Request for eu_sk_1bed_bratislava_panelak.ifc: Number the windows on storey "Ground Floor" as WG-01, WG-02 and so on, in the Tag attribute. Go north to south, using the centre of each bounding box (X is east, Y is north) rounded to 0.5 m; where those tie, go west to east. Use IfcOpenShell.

First a look at what the model holds.

```python
import ifcopenshell
import ifcopenshell.util.element
import ifcopenshell.util.placement

model = ifcopenshell.open("eu_sk_1bed_bratislava_panelak.ifc")
print(model.schema)
storey = next(s for s in model.by_type("IfcBuildingStorey") if s.Name == "Ground Floor")
windows = [e for e in ifcopenshell.util.element.get_decomposition(storey) if e.is_a("IfcWindow")]
for e in sorted(windows, key=lambda e: e.id()):
    origin = ifcopenshell.util.placement.get_local_placement(e.ObjectPlacement)[:3, 3]
    print(e.id(), e.Tag, e.Name, origin.round(2) + 0.0, sep=" | ")
```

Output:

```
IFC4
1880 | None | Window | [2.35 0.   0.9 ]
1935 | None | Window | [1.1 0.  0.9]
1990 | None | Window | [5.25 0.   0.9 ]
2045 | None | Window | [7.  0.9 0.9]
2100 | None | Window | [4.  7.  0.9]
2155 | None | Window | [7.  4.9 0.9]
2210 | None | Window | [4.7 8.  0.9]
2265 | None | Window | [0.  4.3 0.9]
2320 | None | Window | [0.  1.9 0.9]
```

```python
import ifcopenshell
import ifcopenshell.geom
import ifcopenshell.util.element
import ifcopenshell.util.shape

model = ifcopenshell.open("eu_sk_1bed_bratislava_panelak.ifc")
settings = ifcopenshell.geom.settings()
settings.set("use-world-coords", True)


def centre(element):
    shape = ifcopenshell.geom.create_shape(settings, element)
    return ifcopenshell.util.shape.get_bbox_centroid(shape.geometry)


storey = next(s for s in model.by_type("IfcBuildingStorey") if s.Name == "Ground Floor")
windows = [e for e in ifcopenshell.util.element.get_decomposition(storey) if e.is_a("IfcWindow")]

# Insertion points can sit at a corner or the storey origin, so sort by the geometry (in metres).
centres = {e: centre(e) for e in windows}
windows.sort(key=lambda e: (-round(centres[e][1] / 0.5), centres[e][0]))

for i, e in enumerate(windows, start=1):
    number = f"WG-{i:02d}"
    e.Tag = number
    print(e.id(), number)

model.write("eu_sk_1bed_bratislava_panelak_edited.ifc")
```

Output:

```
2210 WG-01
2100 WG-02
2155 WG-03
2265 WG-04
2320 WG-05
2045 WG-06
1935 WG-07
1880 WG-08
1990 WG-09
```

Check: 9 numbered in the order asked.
